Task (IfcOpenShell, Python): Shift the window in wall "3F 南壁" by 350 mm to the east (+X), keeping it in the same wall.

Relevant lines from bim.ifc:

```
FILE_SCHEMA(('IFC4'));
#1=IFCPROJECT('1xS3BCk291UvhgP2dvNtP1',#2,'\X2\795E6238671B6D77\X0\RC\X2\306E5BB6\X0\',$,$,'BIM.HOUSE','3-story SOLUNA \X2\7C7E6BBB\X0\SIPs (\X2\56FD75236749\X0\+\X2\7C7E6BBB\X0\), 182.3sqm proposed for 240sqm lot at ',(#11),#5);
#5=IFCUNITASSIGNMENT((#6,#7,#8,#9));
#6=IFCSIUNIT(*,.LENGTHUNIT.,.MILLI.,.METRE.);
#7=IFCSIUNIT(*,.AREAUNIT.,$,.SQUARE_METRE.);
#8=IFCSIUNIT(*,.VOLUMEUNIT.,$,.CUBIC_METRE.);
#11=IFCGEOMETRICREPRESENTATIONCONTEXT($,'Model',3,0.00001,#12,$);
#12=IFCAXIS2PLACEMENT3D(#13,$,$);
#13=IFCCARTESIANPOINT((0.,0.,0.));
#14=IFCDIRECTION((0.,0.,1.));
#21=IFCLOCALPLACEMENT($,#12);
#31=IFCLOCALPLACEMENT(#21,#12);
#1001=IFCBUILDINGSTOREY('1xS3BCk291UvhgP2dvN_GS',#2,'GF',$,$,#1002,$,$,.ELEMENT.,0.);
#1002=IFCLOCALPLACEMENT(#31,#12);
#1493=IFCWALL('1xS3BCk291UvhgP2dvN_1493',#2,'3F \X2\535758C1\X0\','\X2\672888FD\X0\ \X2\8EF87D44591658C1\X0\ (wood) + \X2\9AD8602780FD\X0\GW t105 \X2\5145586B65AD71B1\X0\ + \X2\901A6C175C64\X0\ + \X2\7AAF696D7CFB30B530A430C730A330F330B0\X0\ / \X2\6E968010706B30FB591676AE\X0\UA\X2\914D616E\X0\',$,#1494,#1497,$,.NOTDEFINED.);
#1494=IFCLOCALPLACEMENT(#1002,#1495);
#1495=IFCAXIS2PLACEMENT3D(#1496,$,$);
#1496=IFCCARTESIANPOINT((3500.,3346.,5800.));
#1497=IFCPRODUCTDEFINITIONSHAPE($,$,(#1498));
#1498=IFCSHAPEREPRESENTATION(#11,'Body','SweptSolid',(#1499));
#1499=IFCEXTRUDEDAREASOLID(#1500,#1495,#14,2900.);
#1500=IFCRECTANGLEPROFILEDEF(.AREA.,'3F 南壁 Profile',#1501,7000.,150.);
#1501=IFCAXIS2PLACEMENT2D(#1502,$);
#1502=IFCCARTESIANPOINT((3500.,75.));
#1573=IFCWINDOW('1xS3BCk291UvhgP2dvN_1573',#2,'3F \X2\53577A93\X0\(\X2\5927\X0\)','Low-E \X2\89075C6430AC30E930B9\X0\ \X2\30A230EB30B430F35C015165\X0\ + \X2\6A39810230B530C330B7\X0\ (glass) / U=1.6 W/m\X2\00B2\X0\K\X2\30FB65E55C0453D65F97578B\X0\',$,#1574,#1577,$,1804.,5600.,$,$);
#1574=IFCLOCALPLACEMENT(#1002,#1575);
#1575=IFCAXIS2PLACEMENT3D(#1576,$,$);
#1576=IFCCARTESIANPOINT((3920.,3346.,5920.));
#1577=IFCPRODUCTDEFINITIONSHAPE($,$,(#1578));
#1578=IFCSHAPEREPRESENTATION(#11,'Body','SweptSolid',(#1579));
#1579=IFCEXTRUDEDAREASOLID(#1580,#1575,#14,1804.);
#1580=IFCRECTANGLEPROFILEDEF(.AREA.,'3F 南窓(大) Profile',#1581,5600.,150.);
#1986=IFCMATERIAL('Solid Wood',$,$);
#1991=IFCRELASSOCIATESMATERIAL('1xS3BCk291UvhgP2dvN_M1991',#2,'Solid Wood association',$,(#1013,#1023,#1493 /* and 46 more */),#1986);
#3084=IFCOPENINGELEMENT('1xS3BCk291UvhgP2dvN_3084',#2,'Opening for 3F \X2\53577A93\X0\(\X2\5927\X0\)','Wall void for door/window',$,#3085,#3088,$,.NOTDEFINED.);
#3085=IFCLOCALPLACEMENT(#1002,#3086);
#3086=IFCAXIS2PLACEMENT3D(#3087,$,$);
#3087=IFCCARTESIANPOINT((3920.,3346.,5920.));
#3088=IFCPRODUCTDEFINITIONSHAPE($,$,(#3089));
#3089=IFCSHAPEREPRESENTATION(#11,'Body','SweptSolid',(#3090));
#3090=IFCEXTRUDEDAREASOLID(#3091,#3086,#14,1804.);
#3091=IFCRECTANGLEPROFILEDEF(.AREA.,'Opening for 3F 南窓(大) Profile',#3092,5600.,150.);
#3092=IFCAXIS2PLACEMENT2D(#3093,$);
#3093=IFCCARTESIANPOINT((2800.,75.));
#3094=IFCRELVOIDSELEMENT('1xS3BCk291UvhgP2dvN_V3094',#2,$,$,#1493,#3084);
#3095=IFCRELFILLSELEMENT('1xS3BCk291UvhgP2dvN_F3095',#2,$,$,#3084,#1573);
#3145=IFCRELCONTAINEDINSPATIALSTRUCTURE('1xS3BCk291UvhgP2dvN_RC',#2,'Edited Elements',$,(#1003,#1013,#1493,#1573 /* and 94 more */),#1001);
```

```python
import ifcopenshell
import ifcopenshell.api.geometry
import ifcopenshell.util.placement
import ifcopenshell.util.unit

model = ifcopenshell.open("bim.ifc")
unit_scale = ifcopenshell.util.unit.calculate_unit_scale(model)

window = model.by_id(1573)
opening = window.FillsVoids[0].RelatingOpeningElement
wall = opening.VoidsElements[0].RelatingBuildingElement

wall_matrix = ifcopenshell.util.placement.get_local_placement(wall.ObjectPlacement)
shift = wall_matrix[:3, 0] * 0.35 / unit_scale
before = ifcopenshell.util.placement.get_local_placement(window.ObjectPlacement)[:3, 3].copy()

# The window is not placed relative to its opening, so move both.
for product in (opening, window):
    matrix = ifcopenshell.util.placement.get_local_placement(product.ObjectPlacement)
    matrix[:3, 3] += shift
    ifcopenshell.api.geometry.edit_object_placement(model, product=product, matrix=matrix, is_si=False)

after = ifcopenshell.util.placement.get_local_placement(window.ObjectPlacement)[:3, 3]
print("window moved by", (after - before).round(3) + 0.0)

model.write("bim_updated.ifc")
```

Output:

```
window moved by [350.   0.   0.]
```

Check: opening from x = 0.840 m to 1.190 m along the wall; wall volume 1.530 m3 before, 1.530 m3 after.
